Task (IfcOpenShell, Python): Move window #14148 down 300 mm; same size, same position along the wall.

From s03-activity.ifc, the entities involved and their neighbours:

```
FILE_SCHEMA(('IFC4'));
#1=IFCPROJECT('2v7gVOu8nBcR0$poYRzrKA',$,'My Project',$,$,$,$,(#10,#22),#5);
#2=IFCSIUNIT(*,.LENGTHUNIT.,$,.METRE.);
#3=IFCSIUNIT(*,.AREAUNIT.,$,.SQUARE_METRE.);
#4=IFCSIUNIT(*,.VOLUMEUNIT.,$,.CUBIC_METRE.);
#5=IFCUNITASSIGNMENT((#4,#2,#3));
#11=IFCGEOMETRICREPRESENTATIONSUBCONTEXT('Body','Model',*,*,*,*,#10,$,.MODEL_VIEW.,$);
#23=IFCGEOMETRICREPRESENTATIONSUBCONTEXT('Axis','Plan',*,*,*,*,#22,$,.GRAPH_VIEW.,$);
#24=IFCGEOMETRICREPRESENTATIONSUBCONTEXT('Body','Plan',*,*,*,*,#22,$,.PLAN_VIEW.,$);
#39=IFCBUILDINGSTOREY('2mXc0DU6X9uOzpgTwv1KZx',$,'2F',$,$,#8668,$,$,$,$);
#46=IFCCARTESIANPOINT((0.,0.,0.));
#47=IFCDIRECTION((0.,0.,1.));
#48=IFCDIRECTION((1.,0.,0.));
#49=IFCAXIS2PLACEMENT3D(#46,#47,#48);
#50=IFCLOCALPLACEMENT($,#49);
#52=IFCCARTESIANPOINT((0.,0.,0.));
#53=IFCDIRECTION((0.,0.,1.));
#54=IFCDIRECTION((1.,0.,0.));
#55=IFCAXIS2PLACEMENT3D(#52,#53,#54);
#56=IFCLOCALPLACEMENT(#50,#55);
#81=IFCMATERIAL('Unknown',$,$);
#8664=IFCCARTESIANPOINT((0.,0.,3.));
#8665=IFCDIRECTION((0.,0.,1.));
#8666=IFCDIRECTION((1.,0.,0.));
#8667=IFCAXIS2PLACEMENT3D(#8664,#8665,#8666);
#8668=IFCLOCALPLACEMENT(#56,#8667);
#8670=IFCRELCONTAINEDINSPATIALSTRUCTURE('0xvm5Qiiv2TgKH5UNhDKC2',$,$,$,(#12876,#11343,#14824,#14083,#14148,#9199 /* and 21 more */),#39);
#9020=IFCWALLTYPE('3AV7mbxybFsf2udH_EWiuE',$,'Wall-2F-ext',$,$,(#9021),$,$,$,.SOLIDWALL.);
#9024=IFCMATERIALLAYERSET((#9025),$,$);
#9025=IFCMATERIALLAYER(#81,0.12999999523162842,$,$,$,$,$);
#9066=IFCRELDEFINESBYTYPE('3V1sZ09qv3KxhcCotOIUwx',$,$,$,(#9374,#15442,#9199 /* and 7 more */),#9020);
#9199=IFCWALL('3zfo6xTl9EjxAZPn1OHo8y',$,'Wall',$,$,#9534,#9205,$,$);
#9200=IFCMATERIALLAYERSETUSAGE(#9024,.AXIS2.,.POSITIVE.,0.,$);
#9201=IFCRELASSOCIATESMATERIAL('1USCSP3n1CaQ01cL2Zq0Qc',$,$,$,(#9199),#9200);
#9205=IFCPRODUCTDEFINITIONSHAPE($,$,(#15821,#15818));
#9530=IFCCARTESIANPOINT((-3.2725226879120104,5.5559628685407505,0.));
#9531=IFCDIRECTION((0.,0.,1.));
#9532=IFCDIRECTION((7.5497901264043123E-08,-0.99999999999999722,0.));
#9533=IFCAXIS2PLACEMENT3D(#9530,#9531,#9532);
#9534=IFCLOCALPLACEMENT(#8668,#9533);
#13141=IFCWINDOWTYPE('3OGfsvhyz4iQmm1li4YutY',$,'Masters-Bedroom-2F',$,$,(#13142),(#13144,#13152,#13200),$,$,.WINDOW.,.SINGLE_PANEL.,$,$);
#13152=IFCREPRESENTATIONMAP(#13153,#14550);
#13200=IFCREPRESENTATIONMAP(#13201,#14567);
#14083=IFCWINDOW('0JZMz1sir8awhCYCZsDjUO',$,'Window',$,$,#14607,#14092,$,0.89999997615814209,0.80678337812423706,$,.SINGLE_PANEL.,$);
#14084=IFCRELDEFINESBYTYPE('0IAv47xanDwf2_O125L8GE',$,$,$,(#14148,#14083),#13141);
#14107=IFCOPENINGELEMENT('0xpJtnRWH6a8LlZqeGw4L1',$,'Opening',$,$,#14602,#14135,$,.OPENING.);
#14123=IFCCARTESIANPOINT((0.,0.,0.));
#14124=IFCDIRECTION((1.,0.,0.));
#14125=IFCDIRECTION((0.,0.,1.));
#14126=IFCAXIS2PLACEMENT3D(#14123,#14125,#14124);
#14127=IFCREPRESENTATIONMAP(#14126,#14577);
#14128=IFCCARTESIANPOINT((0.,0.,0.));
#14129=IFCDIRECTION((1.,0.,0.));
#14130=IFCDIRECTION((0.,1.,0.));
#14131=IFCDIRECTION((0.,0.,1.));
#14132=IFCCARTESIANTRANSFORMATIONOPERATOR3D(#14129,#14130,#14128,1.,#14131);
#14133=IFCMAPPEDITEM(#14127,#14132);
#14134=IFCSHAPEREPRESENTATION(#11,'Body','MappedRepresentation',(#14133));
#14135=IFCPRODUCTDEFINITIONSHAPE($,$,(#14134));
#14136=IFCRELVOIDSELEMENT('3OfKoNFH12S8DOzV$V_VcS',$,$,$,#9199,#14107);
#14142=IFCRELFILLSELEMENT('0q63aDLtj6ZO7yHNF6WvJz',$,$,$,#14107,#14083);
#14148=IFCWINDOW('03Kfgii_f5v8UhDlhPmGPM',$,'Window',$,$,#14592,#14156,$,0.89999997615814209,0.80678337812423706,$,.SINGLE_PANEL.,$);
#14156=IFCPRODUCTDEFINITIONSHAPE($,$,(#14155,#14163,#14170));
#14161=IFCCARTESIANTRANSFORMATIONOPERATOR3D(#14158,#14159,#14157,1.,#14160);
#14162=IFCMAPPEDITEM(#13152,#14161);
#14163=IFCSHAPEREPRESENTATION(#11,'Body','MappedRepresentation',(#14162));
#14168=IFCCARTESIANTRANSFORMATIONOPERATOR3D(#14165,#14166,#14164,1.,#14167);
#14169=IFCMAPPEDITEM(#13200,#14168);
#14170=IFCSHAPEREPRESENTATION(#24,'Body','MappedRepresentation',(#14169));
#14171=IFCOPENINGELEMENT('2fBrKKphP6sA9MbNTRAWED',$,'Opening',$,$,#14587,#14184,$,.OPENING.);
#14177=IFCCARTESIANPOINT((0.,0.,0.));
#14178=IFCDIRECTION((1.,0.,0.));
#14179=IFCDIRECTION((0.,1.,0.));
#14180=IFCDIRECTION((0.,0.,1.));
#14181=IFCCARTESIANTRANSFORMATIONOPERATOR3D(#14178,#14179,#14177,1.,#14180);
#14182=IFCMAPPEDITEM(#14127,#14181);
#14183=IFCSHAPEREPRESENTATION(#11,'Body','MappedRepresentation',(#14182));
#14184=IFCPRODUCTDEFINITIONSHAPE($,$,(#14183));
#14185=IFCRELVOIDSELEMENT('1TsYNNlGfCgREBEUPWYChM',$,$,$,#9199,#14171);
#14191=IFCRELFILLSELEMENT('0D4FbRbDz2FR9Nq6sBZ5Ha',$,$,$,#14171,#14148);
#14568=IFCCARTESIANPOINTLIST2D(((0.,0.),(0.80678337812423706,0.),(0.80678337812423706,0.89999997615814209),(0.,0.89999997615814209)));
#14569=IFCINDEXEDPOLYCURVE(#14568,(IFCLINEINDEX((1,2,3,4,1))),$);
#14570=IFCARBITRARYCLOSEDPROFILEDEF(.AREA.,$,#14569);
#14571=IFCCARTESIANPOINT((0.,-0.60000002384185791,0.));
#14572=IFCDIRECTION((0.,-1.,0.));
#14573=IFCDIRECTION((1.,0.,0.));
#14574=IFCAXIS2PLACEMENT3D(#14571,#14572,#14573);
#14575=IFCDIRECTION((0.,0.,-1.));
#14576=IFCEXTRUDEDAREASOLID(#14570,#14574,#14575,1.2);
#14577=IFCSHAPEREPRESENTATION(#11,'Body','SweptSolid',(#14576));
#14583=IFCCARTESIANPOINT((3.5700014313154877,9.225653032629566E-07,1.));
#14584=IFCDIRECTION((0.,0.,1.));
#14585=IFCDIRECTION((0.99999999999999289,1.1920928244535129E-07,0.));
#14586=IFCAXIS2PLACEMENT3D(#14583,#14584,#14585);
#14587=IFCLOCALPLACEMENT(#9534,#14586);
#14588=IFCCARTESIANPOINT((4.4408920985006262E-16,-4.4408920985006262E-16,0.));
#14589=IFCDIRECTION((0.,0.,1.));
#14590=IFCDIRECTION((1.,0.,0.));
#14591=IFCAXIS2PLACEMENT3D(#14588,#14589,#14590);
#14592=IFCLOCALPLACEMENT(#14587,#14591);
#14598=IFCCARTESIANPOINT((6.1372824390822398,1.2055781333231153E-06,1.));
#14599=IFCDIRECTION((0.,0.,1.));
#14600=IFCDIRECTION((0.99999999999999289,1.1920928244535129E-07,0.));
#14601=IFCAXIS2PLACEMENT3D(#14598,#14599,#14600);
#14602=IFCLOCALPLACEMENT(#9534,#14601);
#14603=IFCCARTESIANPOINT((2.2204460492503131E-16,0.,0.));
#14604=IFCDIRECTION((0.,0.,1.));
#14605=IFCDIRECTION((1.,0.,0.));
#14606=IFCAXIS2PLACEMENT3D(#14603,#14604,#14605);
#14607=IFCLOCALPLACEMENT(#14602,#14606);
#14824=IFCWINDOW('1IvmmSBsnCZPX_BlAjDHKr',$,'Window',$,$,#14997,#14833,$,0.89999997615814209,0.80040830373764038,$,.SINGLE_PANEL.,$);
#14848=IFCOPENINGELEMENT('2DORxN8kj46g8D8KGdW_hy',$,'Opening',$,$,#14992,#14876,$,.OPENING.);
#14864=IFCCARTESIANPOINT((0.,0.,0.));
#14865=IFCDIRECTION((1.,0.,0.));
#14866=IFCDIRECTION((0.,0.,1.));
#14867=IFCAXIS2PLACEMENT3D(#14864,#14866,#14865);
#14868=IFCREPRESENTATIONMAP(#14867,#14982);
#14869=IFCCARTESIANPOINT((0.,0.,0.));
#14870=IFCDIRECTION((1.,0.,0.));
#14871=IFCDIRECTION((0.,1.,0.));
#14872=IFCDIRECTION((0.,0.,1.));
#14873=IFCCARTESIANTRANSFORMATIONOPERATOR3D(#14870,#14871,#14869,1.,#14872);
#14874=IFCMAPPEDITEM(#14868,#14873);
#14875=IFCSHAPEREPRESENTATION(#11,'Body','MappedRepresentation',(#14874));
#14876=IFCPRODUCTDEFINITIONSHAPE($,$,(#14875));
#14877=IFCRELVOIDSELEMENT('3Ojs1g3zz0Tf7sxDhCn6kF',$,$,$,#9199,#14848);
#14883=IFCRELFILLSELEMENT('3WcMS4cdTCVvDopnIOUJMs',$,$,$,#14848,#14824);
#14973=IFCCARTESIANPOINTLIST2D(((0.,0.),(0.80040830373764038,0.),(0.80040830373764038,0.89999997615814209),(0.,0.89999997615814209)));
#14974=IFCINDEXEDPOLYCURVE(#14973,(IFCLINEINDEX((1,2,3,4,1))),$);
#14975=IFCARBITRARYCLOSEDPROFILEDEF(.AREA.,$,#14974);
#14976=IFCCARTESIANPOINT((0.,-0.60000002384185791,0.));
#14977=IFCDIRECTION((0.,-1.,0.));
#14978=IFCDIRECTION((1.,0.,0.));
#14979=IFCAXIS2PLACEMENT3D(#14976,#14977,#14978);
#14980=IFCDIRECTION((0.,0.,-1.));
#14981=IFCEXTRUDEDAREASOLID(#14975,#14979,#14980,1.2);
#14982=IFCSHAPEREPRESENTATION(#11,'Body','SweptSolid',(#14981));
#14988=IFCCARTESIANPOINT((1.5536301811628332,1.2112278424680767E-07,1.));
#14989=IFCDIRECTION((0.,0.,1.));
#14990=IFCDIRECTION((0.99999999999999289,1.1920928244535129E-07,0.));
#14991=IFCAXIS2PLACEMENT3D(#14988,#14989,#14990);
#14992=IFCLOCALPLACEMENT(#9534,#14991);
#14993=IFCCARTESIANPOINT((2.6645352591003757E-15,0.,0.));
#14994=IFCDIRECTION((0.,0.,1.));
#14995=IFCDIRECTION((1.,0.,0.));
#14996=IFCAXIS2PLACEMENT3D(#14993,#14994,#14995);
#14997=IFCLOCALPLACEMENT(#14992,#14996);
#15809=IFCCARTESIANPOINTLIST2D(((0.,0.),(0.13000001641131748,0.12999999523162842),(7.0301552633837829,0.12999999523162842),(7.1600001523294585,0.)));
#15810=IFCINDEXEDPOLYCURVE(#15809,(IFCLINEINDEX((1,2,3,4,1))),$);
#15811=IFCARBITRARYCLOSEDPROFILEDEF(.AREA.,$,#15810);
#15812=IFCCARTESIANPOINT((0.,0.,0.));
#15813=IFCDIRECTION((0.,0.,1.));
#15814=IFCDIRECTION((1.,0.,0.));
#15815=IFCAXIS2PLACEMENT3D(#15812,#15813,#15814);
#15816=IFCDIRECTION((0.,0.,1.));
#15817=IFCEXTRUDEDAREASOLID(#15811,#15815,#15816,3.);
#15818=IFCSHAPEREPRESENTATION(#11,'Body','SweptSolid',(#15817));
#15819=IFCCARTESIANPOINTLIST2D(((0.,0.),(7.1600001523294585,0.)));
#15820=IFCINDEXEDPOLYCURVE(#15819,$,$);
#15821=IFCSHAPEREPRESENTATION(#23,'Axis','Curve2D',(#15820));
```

```python
import numpy as np
import ifcopenshell
import ifcopenshell.api.geometry
import ifcopenshell.util.placement
import ifcopenshell.util.unit

model = ifcopenshell.open("s03-activity.ifc")
unit_scale = ifcopenshell.util.unit.calculate_unit_scale(model)

window = model.by_guid("03Kfgii_f5v8UhDlhPmGPM")
opening = window.FillsVoids[0].RelatingOpeningElement
dz = -0.3 / unit_scale

shift = np.array([0.0, 0.0, dz])
# The window is placed relative to its opening, so it follows when the opening moves.
matrix = ifcopenshell.util.placement.get_local_placement(opening.ObjectPlacement)
matrix[:3, 3] += shift
ifcopenshell.api.geometry.edit_object_placement(
    model, product=opening, matrix=matrix, is_si=False, should_transform_children=True
)

print(f"moved by {dz * unit_scale:+.3f} m")

model.write("s03-activity_rev.ifc")
```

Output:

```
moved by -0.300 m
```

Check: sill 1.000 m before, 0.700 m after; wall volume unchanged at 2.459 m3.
